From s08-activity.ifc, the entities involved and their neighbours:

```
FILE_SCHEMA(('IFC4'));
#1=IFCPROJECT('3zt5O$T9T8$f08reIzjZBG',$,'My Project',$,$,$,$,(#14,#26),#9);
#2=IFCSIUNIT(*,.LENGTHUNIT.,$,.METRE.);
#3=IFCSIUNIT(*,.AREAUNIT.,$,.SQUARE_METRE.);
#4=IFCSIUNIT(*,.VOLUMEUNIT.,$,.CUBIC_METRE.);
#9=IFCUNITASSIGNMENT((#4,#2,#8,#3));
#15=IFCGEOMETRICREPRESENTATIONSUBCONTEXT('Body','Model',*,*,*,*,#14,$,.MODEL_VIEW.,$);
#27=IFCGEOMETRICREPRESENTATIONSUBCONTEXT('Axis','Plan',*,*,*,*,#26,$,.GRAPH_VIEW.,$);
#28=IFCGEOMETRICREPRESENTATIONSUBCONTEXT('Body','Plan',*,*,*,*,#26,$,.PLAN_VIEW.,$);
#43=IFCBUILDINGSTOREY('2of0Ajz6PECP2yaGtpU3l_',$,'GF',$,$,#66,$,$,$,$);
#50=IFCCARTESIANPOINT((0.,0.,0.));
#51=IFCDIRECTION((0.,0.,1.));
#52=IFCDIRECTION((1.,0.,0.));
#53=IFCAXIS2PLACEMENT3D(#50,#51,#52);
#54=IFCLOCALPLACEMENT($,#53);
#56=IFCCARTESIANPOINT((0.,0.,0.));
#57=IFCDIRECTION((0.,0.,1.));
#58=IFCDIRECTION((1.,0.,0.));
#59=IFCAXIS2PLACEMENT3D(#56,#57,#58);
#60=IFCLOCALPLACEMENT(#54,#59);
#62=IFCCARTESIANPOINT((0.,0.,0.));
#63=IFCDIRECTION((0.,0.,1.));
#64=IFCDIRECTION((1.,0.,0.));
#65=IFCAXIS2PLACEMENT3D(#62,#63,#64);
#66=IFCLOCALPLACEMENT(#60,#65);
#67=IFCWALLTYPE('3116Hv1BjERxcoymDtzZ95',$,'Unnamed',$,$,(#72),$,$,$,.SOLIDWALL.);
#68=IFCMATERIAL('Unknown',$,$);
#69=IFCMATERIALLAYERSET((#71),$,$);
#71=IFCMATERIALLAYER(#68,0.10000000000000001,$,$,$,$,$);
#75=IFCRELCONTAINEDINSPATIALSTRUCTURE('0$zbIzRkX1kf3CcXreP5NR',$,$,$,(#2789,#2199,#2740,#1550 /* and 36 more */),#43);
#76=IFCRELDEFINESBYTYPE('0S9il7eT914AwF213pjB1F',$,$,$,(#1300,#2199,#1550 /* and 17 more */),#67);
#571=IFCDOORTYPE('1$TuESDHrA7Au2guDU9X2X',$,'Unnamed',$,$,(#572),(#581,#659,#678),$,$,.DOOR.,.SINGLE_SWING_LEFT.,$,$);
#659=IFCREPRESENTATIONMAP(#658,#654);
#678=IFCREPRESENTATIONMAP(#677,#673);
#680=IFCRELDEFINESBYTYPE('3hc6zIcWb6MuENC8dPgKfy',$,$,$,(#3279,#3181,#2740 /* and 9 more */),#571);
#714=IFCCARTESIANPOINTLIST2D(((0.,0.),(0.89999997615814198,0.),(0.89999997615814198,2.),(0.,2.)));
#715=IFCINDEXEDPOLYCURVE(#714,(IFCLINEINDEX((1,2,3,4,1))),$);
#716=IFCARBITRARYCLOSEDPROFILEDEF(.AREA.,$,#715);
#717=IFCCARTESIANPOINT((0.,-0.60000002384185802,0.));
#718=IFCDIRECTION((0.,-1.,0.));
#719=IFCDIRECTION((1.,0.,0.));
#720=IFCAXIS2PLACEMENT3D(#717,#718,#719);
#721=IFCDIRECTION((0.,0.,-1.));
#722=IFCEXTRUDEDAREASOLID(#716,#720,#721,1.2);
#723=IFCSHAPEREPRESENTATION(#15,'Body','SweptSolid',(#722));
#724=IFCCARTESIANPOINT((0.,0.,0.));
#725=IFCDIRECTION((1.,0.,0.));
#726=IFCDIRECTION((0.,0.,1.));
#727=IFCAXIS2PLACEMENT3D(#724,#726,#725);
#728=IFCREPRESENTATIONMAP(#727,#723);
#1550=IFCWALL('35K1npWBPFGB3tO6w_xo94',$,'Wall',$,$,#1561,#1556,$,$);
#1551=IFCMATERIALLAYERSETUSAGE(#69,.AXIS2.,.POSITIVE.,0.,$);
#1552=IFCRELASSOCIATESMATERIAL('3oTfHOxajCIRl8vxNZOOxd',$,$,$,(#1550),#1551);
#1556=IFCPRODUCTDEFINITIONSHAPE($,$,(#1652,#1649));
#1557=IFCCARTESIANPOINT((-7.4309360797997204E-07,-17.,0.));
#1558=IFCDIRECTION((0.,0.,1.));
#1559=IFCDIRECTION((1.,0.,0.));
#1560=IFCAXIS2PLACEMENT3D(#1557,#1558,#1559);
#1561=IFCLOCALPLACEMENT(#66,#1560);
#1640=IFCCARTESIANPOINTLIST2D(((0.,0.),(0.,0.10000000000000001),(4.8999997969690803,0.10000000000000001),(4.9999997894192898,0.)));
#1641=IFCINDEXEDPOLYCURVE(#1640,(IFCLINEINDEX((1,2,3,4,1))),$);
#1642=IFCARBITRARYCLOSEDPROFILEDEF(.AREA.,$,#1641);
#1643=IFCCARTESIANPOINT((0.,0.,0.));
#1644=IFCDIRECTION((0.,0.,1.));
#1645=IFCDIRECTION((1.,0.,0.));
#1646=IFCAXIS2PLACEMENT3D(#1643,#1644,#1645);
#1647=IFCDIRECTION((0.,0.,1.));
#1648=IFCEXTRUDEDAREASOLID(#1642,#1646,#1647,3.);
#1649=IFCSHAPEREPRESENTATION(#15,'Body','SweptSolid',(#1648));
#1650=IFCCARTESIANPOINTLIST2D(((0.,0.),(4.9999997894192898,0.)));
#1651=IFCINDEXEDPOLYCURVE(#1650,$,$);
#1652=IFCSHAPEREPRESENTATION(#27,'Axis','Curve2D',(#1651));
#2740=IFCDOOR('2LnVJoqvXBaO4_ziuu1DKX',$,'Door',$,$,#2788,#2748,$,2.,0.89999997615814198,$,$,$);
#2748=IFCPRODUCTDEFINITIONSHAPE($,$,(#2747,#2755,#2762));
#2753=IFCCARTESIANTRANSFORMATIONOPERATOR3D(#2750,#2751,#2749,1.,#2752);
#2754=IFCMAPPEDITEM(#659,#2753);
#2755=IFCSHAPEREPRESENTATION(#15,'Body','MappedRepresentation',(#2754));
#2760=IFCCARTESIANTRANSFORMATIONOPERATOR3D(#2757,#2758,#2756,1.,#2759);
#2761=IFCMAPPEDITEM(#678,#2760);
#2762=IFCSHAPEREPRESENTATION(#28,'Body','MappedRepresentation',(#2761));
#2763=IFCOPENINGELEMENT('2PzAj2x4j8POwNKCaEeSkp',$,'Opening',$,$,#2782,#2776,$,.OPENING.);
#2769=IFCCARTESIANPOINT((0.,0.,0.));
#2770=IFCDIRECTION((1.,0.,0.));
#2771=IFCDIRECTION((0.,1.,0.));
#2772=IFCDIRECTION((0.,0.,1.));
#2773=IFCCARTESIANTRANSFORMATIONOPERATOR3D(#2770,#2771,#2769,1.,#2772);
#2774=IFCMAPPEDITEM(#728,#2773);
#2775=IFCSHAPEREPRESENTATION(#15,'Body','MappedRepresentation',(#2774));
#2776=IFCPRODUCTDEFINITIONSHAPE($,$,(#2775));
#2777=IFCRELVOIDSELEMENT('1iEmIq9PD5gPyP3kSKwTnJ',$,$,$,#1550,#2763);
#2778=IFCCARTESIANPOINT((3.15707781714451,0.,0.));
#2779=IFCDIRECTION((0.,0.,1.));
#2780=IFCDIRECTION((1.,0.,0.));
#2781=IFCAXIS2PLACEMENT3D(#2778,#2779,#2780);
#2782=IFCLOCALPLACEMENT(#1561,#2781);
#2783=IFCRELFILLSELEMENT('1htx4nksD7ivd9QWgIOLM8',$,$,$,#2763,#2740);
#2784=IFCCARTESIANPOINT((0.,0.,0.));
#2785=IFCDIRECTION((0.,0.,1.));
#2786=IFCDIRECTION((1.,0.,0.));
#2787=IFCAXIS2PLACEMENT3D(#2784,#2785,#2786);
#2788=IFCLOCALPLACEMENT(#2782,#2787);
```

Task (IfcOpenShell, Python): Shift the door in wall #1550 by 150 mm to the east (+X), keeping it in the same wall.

```python
import ifcopenshell
import ifcopenshell.api.geometry
import ifcopenshell.util.placement
import ifcopenshell.util.unit

model = ifcopenshell.open("s08-activity.ifc")
unit_scale = ifcopenshell.util.unit.calculate_unit_scale(model)

door = model.by_guid("2LnVJoqvXBaO4_ziuu1DKX")
opening = door.FillsVoids[0].RelatingOpeningElement
wall = opening.VoidsElements[0].RelatingBuildingElement

wall_matrix = ifcopenshell.util.placement.get_local_placement(wall.ObjectPlacement)
shift = wall_matrix[:3, 0] * 0.15 / unit_scale
before = ifcopenshell.util.placement.get_local_placement(door.ObjectPlacement)[:3, 3].copy()

# The door is placed relative to its opening, so it follows when the opening moves.
matrix = ifcopenshell.util.placement.get_local_placement(opening.ObjectPlacement)
matrix[:3, 3] += shift
ifcopenshell.api.geometry.edit_object_placement(
    model, product=opening, matrix=matrix, is_si=False, should_transform_children=True
)

after = ifcopenshell.util.placement.get_local_placement(door.ObjectPlacement)[:3, 3]
print("door moved by", (after - before).round(3) + 0.0)

model.write("s08-activity_rev.ifc")
```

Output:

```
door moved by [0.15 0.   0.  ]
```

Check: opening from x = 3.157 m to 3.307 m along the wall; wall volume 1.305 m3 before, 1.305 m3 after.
